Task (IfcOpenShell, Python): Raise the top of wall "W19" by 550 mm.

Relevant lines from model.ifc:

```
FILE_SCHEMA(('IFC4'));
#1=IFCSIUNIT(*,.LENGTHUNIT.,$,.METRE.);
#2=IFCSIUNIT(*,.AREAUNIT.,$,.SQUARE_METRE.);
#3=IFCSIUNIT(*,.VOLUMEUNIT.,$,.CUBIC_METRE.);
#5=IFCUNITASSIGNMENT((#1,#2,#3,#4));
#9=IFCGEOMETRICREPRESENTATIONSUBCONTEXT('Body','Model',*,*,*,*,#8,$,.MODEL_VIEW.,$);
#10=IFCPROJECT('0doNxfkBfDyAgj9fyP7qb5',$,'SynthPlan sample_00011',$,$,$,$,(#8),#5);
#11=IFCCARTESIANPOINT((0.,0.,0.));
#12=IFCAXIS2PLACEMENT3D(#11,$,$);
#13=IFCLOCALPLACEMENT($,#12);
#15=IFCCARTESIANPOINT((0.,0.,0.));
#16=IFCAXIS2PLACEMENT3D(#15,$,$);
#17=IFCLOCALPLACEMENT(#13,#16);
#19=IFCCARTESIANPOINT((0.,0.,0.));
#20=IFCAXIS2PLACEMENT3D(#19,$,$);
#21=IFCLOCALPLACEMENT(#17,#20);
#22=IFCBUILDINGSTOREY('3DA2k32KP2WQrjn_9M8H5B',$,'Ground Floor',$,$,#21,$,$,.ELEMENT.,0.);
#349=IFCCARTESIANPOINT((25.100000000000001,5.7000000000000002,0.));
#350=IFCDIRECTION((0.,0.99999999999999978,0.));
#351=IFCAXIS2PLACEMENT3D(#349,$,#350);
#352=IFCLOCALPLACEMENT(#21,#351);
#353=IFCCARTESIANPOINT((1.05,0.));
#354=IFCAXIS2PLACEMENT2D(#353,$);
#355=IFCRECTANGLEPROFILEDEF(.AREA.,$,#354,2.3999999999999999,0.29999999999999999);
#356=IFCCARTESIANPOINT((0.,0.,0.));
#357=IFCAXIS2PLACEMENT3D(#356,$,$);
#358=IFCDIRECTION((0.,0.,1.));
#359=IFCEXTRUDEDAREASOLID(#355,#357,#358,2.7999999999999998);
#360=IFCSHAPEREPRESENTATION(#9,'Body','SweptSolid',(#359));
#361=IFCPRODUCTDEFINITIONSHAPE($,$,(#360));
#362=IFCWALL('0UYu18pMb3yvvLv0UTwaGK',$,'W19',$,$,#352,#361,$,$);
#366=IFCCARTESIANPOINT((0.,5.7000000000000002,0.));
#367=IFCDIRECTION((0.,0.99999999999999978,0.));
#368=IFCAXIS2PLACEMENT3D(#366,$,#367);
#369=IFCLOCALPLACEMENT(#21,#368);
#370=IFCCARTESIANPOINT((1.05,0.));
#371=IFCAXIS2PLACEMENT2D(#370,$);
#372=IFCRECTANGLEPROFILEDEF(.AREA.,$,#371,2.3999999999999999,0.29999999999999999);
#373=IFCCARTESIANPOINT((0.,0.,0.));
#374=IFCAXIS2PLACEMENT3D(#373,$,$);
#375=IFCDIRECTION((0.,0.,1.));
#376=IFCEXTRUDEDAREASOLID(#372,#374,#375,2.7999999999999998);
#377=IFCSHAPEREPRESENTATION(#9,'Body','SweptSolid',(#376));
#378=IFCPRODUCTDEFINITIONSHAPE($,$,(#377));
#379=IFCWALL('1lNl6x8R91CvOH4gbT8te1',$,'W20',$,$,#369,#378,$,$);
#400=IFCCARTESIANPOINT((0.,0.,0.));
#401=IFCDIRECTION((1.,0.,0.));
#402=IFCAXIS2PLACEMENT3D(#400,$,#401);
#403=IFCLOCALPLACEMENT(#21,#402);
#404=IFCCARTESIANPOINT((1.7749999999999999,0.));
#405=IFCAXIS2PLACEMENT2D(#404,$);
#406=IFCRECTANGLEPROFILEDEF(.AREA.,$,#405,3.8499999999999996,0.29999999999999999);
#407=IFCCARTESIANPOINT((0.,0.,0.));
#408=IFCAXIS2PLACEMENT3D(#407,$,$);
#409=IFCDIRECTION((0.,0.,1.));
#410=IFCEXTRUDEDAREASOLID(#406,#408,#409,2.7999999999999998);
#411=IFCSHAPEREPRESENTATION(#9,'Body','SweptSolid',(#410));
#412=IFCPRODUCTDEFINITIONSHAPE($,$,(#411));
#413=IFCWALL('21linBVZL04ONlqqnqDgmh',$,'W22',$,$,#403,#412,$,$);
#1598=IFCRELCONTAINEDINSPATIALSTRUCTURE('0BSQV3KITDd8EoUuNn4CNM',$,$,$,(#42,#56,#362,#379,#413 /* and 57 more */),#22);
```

```python
import ifcopenshell
import ifcopenshell.geom
import ifcopenshell.util.representation
import ifcopenshell.util.shape
import ifcopenshell.util.unit

model = ifcopenshell.open("model.ifc")
unit_scale = ifcopenshell.util.unit.calculate_unit_scale(model)
settings = ifcopenshell.geom.settings()


def volume(element):
    """Net volume in cubic metres, openings subtracted."""
    shape = ifcopenshell.geom.create_shape(settings, element)
    return ifcopenshell.util.shape.get_volume(shape.geometry)


wall = model.by_guid("0UYu18pMb3yvvLv0UTwaGK")
before = volume(wall)

body = ifcopenshell.util.representation.get_representation(wall, "Model", "Body")
solid = body.Items[0]
old_height = solid.Depth
solid.Depth += 0.55 / unit_scale
after = volume(wall)

print(f"height {old_height:g} -> {solid.Depth:g}, volume {before:.3f} -> {after:.3f} m3")

model.write("model_edited.ifc")
```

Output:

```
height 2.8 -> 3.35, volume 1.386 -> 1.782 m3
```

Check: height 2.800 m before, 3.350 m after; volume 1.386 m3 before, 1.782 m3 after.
